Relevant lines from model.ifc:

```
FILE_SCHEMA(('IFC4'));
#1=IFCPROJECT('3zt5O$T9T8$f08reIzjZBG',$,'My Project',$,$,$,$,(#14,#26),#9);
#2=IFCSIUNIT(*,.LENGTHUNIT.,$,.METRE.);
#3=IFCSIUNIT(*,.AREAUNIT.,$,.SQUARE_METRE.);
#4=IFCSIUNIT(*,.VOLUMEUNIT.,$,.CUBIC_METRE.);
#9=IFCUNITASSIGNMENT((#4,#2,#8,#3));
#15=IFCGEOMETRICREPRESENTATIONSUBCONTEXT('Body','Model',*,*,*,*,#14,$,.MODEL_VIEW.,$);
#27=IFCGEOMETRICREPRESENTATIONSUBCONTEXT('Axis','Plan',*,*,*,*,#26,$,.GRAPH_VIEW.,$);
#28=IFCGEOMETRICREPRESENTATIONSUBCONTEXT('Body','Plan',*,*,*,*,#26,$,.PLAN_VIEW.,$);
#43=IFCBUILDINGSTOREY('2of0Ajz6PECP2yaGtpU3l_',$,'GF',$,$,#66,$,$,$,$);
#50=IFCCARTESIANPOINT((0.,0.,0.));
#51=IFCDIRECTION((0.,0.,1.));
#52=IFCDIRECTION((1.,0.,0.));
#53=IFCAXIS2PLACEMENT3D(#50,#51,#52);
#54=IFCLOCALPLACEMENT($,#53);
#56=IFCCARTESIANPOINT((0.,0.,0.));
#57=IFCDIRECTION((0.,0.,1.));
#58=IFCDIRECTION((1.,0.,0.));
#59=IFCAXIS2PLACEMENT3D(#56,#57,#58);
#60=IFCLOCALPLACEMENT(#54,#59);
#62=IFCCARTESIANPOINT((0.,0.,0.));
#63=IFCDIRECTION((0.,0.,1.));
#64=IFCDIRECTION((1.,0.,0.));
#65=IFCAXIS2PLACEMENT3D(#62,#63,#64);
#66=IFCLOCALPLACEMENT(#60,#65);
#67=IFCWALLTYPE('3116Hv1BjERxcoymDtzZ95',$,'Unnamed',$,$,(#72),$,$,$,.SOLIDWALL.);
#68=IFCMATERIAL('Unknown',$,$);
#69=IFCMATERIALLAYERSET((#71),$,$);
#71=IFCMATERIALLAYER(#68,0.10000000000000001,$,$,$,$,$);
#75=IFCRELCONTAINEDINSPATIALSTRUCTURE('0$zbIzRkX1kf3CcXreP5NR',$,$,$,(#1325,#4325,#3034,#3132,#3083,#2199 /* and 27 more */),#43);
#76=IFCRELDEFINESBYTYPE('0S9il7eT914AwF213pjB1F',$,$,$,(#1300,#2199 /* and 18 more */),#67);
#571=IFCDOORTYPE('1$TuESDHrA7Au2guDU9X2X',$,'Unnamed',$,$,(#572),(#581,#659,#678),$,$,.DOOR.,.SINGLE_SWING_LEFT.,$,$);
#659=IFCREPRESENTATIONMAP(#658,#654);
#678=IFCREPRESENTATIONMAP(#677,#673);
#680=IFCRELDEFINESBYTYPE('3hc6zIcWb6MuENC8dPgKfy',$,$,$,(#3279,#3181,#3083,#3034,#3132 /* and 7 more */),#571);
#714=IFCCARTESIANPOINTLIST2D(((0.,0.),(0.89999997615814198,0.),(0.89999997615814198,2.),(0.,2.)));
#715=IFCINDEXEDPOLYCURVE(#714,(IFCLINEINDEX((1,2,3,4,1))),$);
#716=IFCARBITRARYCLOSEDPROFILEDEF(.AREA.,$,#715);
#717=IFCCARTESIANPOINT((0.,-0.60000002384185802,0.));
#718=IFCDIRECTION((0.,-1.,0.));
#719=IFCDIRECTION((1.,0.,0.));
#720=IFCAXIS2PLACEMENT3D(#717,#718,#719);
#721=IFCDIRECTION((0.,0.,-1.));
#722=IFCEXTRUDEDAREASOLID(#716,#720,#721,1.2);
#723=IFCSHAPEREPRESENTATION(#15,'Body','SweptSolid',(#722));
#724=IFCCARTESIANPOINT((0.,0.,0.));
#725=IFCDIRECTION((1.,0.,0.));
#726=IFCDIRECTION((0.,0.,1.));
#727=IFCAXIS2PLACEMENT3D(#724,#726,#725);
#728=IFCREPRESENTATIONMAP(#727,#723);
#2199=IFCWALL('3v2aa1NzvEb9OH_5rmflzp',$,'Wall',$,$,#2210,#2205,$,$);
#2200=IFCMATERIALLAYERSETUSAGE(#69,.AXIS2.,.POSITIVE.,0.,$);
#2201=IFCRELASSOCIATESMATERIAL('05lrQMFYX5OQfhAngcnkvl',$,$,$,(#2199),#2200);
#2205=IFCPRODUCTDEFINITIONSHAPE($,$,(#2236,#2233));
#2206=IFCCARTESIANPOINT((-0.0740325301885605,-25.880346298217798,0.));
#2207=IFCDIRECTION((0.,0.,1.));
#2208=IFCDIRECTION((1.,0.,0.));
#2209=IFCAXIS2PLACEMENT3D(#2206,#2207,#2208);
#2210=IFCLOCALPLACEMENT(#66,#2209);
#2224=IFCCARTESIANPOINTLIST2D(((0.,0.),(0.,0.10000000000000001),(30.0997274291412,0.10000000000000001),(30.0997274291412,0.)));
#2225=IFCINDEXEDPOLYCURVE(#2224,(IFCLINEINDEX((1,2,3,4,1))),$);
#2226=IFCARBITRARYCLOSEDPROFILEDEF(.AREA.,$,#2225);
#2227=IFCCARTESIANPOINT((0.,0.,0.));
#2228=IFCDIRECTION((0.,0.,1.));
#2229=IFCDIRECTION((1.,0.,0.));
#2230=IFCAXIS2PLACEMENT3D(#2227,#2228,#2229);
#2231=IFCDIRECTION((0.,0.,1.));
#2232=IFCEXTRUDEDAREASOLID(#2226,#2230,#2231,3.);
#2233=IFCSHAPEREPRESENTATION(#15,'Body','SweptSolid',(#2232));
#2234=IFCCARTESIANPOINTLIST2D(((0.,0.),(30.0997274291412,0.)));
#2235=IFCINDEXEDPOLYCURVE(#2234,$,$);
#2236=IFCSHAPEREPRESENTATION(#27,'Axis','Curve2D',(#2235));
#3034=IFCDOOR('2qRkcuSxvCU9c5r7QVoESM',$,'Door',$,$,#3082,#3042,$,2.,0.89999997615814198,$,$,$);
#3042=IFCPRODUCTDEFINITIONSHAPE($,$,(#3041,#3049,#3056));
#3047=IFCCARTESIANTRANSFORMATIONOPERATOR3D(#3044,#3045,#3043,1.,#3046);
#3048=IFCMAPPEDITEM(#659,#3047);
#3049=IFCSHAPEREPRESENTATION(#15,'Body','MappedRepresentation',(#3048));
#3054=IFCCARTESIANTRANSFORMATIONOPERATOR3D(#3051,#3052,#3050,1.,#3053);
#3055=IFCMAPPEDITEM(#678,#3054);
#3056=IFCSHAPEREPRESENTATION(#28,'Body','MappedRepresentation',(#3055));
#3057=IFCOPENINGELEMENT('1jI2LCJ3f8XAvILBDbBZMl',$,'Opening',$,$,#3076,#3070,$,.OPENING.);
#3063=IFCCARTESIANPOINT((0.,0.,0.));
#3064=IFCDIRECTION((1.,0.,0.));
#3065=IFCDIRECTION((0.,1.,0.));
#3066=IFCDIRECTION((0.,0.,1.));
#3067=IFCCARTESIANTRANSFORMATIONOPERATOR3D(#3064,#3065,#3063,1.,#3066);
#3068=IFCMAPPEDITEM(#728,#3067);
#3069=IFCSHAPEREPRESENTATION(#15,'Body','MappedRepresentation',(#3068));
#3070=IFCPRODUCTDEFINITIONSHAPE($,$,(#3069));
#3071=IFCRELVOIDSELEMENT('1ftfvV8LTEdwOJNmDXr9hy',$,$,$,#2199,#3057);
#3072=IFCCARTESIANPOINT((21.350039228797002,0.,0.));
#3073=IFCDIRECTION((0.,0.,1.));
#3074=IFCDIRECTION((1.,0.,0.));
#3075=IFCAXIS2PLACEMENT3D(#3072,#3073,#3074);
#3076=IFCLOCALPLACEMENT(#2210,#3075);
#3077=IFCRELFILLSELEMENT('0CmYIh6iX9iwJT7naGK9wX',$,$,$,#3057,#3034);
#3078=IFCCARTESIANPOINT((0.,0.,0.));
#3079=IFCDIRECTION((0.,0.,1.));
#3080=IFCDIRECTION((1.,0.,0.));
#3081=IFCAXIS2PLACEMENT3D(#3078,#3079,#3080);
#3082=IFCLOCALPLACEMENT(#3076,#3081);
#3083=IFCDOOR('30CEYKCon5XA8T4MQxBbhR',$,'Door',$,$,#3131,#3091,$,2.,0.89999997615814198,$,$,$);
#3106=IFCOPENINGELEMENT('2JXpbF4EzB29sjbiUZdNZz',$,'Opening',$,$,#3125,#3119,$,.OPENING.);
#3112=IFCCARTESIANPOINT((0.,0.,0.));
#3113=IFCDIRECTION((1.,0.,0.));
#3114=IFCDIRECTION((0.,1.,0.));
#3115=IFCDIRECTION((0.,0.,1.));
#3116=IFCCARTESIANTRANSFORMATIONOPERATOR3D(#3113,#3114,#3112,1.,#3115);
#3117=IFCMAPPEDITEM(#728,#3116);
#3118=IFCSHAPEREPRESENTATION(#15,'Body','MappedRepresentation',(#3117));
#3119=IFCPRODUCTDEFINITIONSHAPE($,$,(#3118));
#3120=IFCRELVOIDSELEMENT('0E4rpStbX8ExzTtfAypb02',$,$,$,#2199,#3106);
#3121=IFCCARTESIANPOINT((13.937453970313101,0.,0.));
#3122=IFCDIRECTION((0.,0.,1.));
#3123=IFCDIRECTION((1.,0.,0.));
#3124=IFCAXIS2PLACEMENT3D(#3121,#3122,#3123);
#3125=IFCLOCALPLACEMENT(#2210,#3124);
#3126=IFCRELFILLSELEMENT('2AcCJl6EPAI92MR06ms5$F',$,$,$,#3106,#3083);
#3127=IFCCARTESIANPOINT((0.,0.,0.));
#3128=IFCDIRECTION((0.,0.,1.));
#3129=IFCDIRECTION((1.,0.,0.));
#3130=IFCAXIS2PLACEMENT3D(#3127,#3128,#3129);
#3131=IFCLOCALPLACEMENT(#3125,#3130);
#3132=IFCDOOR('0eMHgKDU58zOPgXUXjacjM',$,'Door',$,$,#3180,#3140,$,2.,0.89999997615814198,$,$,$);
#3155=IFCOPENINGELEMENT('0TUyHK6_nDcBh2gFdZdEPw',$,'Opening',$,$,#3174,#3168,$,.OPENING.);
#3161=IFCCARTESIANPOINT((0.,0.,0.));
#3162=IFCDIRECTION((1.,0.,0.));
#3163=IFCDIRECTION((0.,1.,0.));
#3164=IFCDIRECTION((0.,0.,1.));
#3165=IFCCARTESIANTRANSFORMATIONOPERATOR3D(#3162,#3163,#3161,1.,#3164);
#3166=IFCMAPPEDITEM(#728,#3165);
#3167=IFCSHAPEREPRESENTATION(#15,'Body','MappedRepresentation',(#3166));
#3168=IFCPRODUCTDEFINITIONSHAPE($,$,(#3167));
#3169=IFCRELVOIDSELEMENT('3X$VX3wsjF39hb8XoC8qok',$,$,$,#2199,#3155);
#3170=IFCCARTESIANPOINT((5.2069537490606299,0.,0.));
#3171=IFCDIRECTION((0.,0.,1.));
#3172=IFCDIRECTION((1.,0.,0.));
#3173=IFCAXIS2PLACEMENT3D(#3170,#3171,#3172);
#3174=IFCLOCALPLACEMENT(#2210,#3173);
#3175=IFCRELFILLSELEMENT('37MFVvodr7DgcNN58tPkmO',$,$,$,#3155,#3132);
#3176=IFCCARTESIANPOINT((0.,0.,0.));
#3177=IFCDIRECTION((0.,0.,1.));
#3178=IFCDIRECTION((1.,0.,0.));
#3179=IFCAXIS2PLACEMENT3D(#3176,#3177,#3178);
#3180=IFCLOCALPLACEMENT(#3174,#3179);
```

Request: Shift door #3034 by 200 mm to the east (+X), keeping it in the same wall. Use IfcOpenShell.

```python
import ifcopenshell
import ifcopenshell.api.geometry
import ifcopenshell.util.placement

model = ifcopenshell.open("model.ifc")

door = model.by_id(3034)
opening = door.FillsVoids[0].RelatingOpeningElement
wall = opening.VoidsElements[0].RelatingBuildingElement

wall_matrix = ifcopenshell.util.placement.get_local_placement(wall.ObjectPlacement)
shift = wall_matrix[:3, 0] * 0.2
before = ifcopenshell.util.placement.get_local_placement(door.ObjectPlacement)[:3, 3].copy()

# The door is placed relative to its opening, so it follows when the opening moves.
matrix = ifcopenshell.util.placement.get_local_placement(opening.ObjectPlacement)
matrix[:3, 3] += shift
ifcopenshell.api.geometry.edit_object_placement(
    model, product=opening, matrix=matrix, is_si=False, should_transform_children=True
)

after = ifcopenshell.util.placement.get_local_placement(door.ObjectPlacement)[:3, 3]
print("door moved by", (after - before).round(3) + 0.0)

model.write("model_updated.ifc")
```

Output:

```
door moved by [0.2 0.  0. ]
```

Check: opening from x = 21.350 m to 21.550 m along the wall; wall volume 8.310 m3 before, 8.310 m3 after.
